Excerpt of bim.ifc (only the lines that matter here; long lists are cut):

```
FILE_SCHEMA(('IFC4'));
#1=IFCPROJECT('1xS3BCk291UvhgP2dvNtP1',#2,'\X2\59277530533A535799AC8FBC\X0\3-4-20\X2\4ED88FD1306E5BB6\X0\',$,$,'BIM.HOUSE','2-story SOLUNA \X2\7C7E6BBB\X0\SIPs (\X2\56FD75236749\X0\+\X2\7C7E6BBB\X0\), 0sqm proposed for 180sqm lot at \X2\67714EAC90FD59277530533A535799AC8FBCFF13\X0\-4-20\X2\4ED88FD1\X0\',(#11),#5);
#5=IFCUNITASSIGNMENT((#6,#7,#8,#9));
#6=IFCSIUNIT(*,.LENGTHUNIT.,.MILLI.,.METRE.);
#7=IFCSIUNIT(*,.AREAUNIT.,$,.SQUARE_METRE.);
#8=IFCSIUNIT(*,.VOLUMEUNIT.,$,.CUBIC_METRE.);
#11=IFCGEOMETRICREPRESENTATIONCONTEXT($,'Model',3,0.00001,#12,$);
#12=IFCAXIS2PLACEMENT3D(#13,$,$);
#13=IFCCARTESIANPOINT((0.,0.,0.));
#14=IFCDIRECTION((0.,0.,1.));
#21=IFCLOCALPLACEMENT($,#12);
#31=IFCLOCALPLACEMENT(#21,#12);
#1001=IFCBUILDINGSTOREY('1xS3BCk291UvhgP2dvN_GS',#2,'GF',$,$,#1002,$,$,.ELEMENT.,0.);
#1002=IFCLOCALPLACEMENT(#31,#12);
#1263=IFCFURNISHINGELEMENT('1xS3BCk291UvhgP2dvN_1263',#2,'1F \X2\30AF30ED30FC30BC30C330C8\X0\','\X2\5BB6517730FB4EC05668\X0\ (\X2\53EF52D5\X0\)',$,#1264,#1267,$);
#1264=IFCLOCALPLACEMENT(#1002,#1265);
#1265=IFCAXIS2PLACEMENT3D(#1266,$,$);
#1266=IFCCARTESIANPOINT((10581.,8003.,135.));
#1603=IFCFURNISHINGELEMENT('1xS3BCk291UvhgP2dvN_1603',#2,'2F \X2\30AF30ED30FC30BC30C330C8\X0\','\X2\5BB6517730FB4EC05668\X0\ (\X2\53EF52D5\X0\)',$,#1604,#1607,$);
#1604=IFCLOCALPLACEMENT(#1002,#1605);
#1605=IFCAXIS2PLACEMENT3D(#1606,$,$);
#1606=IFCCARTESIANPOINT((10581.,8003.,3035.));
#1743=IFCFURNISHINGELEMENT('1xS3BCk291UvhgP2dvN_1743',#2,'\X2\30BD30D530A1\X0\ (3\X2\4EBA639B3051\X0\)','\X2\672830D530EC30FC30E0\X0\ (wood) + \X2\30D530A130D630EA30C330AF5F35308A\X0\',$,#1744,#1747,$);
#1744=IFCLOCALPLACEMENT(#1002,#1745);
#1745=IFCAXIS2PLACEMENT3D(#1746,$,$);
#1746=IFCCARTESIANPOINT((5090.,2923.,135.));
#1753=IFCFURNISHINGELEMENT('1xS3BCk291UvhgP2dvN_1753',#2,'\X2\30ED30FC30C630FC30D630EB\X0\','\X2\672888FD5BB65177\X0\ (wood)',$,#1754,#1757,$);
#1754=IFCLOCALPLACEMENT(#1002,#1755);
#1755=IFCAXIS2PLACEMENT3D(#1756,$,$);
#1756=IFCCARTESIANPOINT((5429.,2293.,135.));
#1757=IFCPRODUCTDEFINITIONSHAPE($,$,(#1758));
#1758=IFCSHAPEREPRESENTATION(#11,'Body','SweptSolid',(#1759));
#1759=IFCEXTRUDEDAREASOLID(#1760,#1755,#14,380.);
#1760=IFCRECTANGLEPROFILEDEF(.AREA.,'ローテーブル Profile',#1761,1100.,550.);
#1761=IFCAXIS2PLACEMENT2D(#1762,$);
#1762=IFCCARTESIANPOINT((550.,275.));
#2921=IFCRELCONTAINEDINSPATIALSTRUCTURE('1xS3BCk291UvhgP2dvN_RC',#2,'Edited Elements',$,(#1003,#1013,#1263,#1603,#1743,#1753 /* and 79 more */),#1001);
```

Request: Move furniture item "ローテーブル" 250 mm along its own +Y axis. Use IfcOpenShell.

```python
import ifcopenshell
import ifcopenshell.api.geometry
import ifcopenshell.util.placement
import ifcopenshell.util.unit

model = ifcopenshell.open("bim.ifc")
unit_scale = ifcopenshell.util.unit.calculate_unit_scale(model)

item = model.by_id(1753)
matrix = ifcopenshell.util.placement.get_local_placement(item.ObjectPlacement)
matrix[:3, 3] += matrix[:3, 1] * 0.25 / unit_scale
ifcopenshell.api.geometry.edit_object_placement(model, product=item, matrix=matrix, is_si=False)

print(ifcopenshell.util.placement.get_local_placement(item.ObjectPlacement).round(3) + 0.0)

model.write("bim_edited.ifc")
```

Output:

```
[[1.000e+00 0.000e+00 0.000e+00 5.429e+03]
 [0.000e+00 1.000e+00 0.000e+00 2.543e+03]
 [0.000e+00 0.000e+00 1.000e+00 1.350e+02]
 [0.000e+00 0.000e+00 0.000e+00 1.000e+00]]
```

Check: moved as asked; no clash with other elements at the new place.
